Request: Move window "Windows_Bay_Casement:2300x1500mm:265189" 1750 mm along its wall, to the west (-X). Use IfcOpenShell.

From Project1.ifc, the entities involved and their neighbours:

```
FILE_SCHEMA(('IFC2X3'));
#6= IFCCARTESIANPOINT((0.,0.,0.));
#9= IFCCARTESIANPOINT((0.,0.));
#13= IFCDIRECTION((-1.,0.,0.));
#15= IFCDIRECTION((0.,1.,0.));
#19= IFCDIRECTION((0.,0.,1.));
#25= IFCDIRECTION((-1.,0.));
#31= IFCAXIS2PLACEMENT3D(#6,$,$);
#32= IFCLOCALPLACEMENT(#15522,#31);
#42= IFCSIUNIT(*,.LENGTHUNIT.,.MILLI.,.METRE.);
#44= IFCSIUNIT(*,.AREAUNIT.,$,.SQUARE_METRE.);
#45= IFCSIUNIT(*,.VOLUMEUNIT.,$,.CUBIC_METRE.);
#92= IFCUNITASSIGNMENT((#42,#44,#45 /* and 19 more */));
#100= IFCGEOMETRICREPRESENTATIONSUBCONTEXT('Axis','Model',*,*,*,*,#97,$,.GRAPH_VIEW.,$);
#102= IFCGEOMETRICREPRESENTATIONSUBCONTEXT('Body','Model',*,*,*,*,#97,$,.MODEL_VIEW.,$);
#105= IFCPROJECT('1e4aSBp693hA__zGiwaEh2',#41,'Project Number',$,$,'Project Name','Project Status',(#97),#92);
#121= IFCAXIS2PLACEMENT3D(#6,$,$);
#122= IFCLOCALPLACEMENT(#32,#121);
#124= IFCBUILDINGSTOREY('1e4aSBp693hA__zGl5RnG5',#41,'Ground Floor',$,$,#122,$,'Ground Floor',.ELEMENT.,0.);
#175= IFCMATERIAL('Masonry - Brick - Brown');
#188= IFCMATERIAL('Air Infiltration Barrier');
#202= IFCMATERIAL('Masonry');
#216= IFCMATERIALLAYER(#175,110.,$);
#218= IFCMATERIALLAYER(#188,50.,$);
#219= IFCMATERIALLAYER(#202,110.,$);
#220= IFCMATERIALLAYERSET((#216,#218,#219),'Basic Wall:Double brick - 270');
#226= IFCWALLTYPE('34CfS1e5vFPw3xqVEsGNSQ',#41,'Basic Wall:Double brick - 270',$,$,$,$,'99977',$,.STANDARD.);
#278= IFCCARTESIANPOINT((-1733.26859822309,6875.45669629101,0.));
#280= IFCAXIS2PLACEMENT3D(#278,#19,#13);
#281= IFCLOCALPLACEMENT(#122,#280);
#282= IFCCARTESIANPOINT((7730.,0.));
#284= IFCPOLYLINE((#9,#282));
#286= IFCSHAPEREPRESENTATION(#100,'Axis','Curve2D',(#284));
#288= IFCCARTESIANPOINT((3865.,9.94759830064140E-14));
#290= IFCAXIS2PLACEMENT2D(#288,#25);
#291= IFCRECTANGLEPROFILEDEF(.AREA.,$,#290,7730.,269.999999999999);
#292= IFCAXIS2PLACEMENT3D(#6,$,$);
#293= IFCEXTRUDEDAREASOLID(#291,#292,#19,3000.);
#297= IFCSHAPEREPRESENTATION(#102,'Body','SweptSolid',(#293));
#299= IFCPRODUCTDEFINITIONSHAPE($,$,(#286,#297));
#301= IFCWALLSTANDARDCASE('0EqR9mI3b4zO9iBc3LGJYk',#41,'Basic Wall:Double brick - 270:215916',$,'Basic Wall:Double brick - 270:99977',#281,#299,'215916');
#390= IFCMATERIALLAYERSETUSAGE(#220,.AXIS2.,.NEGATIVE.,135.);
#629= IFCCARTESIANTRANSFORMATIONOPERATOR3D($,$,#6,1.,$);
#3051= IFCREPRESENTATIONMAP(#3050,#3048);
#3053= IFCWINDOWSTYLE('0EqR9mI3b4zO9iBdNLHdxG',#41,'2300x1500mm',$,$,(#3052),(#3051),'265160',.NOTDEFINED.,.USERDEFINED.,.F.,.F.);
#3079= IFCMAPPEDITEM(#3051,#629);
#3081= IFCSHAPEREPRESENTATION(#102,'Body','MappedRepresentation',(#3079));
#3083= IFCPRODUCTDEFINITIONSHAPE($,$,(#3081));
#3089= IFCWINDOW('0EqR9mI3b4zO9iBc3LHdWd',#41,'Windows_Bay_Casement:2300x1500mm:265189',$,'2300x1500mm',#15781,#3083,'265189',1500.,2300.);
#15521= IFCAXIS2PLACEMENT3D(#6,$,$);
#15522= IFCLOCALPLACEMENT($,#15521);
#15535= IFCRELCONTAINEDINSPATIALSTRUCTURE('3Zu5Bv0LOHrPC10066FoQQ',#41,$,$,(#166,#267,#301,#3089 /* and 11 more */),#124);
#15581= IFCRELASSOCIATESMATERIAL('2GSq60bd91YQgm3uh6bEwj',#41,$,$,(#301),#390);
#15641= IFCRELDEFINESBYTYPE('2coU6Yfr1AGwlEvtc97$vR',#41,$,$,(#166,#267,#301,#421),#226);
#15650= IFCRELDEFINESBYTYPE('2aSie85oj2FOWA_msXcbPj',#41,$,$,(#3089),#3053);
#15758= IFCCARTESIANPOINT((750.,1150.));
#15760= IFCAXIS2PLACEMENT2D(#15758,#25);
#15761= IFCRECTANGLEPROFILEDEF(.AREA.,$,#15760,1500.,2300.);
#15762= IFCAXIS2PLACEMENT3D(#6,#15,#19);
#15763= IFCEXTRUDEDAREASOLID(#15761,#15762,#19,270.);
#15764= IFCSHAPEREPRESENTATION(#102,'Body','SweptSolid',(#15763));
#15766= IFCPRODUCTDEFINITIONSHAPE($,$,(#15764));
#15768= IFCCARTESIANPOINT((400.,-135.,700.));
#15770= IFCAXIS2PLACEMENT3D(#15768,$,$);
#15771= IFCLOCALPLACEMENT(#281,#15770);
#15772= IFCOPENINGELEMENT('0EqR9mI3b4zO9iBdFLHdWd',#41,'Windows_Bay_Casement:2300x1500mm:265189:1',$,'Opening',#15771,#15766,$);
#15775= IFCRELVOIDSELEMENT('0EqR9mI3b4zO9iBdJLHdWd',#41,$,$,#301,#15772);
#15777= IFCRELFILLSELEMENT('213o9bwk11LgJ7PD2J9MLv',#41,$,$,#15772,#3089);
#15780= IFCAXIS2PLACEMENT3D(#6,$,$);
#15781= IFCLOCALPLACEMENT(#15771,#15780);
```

```python
import ifcopenshell
import ifcopenshell.api.geometry
import ifcopenshell.util.placement
import ifcopenshell.util.unit

model = ifcopenshell.open("Project1.ifc")
unit_scale = ifcopenshell.util.unit.calculate_unit_scale(model)

window = model.by_guid("0EqR9mI3b4zO9iBc3LHdWd")
opening = window.FillsVoids[0].RelatingOpeningElement
wall = opening.VoidsElements[0].RelatingBuildingElement

wall_matrix = ifcopenshell.util.placement.get_local_placement(wall.ObjectPlacement)
shift = wall_matrix[:3, 0] * 1.75 / unit_scale
before = ifcopenshell.util.placement.get_local_placement(window.ObjectPlacement)[:3, 3].copy()

# The window is placed relative to its opening, so it follows when the opening moves.
matrix = ifcopenshell.util.placement.get_local_placement(opening.ObjectPlacement)
matrix[:3, 3] += shift
ifcopenshell.api.geometry.edit_object_placement(
    model, product=opening, matrix=matrix, is_si=False, should_transform_children=True
)

after = ifcopenshell.util.placement.get_local_placement(window.ObjectPlacement)[:3, 3]
print("window moved by", (after - before).round(3) + 0.0)

model.write("Project1-out.ifc")
```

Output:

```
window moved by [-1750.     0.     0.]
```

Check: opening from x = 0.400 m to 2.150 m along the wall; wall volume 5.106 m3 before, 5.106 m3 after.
